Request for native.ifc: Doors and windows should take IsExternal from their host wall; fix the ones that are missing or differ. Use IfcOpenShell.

First a look at what the model holds.

```python
import ifcopenshell
import ifcopenshell.util.element

model = ifcopenshell.open("native.ifc")
print(model.schema)
seen = {}
for e in model.by_type("IfcDoor") + model.by_type("IfcWindow"):
    if not e.FillsVoids:
        continue
    host = e.FillsVoids[0].RelatingOpeningElement.VoidsElements[0].RelatingBuildingElement
    own = ifcopenshell.util.element.get_pset(e, f"Pset_{e.is_a()[3:].removesuffix('StandardCase')}Common", "IsExternal")
    wall = ifcopenshell.util.element.get_pset(host, "Pset_WallCommon", "IsExternal")
    seen[e.is_a(), own, wall] = seen.get((e.is_a(), own, wall), 0) + 1
for (cls, own, wall), count in sorted(seen.items(), key=str):
    print(count, cls, "IsExternal:", own, "| host wall:", wall)
```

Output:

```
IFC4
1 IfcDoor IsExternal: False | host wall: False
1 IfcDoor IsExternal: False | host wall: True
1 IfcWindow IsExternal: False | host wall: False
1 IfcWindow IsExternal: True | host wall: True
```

```python
import ifcopenshell
import ifcopenshell.api.pset
import ifcopenshell.util.element

model = ifcopenshell.open("native.ifc")

count = 0
for ifc_class, pset_name in (("IfcDoor", "Pset_DoorCommon"), ("IfcWindow", "Pset_WindowCommon")):
    for e in model.by_type(ifc_class):
        if not e.FillsVoids:
            continue
        host = e.FillsVoids[0].RelatingOpeningElement.VoidsElements[0].RelatingBuildingElement
        external = ifcopenshell.util.element.get_pset(host, "Pset_WallCommon", "IsExternal")
        if external is None or ifcopenshell.util.element.get_pset(e, pset_name, "IsExternal") == external:
            continue
        pset = ifcopenshell.api.pset.add_pset(model, product=e, name=pset_name)
        ifcopenshell.api.pset.edit_pset(model, pset=pset, properties={"IsExternal": external})
        count += 1

print(count, "updated")

model.write("native-out.ifc")
```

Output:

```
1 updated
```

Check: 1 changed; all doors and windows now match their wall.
